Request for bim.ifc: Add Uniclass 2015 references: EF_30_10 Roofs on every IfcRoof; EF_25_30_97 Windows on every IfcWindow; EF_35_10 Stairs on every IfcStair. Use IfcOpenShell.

First a look at what the model holds.

```python
import ifcopenshell

model = ifcopenshell.open("bim.ifc")
print(model.schema)
print("classifications:", [c.Name for c in model.by_type("IfcClassification")])
for ifc_class in ("IfcDoor", "IfcRoof", "IfcStair", "IfcWall", "IfcWindow"):
    print(ifc_class, len(model.by_type(ifc_class)))
```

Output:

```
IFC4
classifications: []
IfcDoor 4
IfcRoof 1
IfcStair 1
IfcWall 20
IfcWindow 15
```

```python
import ifcopenshell
import ifcopenshell.api.classification

model = ifcopenshell.open("bim.ifc")

system = ifcopenshell.api.classification.add_classification(model, classification="Uniclass 2015")

codes = {
    "IfcRoof": ("EF_30_10", "Roofs"),
    "IfcWindow": ("EF_25_30_97", "Windows"),
    "IfcStair": ("EF_35_10", "Stairs"),
}
for ifc_class, (code, name) in codes.items():
    products = model.by_type(ifc_class)
    ifcopenshell.api.classification.add_reference(
        model, products=products, classification=system, identification=code, name=name
    )
    print(code, len(products))

model.write("bim-out.ifc")
```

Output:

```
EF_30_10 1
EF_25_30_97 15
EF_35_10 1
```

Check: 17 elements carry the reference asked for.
